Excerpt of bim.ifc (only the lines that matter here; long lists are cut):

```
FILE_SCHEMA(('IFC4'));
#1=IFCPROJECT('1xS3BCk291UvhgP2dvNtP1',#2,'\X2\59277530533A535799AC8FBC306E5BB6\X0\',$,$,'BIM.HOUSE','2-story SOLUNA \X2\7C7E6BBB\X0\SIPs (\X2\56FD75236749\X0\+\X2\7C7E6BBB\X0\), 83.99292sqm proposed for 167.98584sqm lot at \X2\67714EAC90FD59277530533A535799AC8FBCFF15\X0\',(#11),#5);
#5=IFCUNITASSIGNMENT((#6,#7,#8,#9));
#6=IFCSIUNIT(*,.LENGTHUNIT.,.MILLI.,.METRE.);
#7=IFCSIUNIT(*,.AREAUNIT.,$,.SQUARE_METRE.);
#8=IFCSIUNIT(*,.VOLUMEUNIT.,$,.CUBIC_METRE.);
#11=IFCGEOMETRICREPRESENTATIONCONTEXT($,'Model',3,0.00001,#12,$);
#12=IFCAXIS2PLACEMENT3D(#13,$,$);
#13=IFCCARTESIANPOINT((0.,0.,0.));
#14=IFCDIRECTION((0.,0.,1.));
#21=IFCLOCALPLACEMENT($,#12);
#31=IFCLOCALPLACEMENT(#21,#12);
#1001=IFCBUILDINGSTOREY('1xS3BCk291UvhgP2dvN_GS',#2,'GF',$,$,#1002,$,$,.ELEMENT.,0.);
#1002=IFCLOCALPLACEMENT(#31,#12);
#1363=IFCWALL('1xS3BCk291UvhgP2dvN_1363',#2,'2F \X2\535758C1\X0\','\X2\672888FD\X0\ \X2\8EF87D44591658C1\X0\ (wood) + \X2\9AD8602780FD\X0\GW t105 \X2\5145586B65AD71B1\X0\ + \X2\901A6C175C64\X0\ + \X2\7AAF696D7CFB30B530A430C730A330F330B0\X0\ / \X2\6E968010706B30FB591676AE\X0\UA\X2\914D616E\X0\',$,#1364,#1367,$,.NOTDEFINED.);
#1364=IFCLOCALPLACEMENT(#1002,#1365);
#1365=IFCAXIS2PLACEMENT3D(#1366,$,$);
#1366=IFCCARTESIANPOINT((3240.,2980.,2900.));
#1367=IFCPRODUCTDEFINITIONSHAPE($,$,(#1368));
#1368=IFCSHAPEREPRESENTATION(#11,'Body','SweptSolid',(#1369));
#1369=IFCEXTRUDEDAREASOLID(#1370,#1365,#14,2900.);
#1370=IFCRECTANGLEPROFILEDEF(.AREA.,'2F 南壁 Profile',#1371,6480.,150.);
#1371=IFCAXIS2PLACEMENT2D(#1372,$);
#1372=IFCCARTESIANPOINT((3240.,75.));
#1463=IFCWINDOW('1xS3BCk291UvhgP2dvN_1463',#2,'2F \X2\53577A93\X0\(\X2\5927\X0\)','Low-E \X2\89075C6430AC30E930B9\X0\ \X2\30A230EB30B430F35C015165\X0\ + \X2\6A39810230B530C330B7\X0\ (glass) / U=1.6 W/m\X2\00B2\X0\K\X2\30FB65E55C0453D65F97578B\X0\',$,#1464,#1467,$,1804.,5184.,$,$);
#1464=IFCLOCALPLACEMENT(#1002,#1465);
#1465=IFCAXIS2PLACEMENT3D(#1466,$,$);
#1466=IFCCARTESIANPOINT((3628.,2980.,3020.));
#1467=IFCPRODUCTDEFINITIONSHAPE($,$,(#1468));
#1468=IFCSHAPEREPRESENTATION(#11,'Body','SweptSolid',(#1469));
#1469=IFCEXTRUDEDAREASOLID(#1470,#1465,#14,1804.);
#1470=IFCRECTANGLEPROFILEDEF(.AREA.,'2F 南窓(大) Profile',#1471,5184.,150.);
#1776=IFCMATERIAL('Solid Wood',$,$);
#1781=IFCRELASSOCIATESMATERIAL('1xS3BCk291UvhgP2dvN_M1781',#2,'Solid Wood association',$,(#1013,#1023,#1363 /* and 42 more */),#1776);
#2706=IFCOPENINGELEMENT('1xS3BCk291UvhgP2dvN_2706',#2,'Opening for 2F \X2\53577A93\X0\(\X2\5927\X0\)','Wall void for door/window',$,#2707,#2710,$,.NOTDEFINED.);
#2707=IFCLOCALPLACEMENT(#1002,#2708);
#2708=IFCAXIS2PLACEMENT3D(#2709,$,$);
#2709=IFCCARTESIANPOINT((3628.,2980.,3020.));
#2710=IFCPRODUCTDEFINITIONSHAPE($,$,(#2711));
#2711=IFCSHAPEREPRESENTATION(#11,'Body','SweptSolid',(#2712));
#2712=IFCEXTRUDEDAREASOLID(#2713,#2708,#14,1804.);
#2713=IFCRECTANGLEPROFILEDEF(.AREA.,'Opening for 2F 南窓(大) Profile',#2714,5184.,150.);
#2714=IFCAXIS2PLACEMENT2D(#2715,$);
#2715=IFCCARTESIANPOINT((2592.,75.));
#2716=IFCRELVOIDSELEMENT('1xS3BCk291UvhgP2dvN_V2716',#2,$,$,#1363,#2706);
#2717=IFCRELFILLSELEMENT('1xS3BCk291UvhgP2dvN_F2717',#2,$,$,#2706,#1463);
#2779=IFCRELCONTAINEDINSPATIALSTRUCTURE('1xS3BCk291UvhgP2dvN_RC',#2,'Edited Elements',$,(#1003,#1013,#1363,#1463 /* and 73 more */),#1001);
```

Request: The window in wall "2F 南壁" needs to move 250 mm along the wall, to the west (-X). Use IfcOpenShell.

```python
import ifcopenshell
import ifcopenshell.api.geometry
import ifcopenshell.util.placement
import ifcopenshell.util.unit

model = ifcopenshell.open("bim.ifc")
unit_scale = ifcopenshell.util.unit.calculate_unit_scale(model)

window = model.by_guid("1xS3BCk291UvhgP2dvN_1463")
opening = window.FillsVoids[0].RelatingOpeningElement
wall = opening.VoidsElements[0].RelatingBuildingElement

wall_matrix = ifcopenshell.util.placement.get_local_placement(wall.ObjectPlacement)
shift = wall_matrix[:3, 0] * -0.25 / unit_scale
before = ifcopenshell.util.placement.get_local_placement(window.ObjectPlacement)[:3, 3].copy()

# The window is not placed relative to its opening, so move both.
for product in (opening, window):
    matrix = ifcopenshell.util.placement.get_local_placement(product.ObjectPlacement)
    matrix[:3, 3] += shift
    ifcopenshell.api.geometry.edit_object_placement(model, product=product, matrix=matrix, is_si=False)

after = ifcopenshell.util.placement.get_local_placement(window.ObjectPlacement)[:3, 3]
print("window moved by", (after - before).round(3) + 0.0)

model.write("bim_rev.ifc")
```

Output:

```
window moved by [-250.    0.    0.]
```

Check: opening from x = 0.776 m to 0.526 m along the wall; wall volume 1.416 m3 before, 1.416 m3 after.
